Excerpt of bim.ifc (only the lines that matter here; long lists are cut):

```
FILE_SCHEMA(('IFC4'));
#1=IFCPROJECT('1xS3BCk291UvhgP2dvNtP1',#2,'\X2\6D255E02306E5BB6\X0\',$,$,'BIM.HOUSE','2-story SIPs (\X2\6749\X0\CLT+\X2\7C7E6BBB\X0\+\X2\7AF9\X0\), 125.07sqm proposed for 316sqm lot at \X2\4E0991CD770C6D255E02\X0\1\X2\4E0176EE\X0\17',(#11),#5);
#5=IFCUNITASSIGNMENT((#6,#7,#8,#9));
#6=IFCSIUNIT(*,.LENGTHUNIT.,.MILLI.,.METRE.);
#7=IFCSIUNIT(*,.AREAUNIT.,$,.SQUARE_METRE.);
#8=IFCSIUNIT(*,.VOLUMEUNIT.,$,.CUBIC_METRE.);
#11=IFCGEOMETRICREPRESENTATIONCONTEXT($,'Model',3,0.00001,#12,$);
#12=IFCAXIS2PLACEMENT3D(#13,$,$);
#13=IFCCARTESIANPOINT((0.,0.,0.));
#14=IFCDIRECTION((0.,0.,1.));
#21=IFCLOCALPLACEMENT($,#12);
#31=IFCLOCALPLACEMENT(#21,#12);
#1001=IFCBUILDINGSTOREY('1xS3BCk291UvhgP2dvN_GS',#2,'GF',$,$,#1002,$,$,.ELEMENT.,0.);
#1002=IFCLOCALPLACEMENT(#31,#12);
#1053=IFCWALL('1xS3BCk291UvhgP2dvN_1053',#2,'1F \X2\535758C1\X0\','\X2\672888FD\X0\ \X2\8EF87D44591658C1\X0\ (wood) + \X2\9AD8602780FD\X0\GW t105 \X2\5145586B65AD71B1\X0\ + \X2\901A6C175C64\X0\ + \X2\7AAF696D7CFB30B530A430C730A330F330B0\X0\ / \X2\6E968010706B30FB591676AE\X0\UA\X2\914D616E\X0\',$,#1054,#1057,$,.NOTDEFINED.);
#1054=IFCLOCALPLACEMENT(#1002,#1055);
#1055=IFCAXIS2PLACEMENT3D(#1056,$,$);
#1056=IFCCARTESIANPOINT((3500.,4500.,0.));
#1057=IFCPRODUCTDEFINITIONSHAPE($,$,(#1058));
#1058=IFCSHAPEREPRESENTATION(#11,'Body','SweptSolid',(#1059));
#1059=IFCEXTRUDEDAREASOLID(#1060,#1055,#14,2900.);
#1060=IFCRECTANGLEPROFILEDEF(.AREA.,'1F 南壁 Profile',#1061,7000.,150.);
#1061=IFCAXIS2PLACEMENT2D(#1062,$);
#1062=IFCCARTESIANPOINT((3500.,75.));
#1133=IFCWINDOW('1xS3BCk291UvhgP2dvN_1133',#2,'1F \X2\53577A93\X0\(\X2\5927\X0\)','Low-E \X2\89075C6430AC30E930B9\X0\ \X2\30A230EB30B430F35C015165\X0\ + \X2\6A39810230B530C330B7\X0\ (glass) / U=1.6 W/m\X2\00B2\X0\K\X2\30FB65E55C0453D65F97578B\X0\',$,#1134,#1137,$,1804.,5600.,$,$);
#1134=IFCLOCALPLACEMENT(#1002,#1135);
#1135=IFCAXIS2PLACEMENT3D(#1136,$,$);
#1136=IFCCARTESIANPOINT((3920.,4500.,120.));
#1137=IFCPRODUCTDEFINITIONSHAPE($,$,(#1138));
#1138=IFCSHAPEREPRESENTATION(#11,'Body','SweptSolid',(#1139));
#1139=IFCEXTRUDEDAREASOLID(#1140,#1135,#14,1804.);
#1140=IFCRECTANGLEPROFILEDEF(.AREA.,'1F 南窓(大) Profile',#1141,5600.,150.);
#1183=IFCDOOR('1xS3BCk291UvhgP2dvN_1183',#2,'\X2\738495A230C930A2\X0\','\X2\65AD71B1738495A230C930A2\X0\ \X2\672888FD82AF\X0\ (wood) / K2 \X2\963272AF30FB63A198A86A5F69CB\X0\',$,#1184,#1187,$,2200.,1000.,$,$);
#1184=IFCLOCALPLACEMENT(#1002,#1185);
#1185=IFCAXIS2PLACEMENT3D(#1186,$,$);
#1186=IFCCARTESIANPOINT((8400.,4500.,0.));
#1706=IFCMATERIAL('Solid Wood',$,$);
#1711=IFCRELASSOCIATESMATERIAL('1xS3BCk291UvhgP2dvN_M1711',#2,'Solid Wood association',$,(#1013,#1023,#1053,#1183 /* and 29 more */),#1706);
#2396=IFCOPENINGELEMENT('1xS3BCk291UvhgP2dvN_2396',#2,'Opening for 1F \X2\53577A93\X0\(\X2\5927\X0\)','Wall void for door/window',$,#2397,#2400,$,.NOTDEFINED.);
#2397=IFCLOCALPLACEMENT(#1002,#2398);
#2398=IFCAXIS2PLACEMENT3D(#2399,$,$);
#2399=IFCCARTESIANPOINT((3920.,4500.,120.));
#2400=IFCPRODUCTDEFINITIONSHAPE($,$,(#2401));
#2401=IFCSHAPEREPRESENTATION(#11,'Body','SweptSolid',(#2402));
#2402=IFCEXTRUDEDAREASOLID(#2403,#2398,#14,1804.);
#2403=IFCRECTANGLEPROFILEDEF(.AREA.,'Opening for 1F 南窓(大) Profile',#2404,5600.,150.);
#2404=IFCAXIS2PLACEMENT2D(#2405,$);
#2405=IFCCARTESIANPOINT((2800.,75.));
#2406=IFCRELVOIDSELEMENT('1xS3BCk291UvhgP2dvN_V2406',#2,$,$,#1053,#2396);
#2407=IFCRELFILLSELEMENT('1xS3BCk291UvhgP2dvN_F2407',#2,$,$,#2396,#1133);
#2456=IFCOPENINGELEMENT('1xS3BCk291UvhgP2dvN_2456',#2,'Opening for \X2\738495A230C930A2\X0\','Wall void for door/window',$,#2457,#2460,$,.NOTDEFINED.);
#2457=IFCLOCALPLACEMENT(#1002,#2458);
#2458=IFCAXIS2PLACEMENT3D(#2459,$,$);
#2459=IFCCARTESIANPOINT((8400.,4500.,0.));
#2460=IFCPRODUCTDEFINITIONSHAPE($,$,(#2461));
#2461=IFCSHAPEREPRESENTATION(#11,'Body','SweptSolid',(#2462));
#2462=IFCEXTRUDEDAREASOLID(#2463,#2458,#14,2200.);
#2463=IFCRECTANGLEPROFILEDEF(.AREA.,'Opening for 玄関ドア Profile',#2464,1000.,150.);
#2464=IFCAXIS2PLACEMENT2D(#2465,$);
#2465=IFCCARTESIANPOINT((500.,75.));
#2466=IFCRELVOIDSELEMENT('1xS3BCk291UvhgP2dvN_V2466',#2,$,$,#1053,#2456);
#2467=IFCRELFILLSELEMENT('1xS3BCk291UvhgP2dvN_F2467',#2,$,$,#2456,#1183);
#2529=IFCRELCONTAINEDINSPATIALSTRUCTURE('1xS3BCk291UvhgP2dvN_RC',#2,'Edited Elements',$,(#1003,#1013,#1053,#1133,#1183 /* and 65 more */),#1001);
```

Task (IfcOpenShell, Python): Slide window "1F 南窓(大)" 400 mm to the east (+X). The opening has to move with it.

```python
import ifcopenshell
import ifcopenshell.api.geometry
import ifcopenshell.util.placement
import ifcopenshell.util.unit

model = ifcopenshell.open("bim.ifc")
unit_scale = ifcopenshell.util.unit.calculate_unit_scale(model)

window = model.by_guid("1xS3BCk291UvhgP2dvN_1133")
opening = window.FillsVoids[0].RelatingOpeningElement
wall = opening.VoidsElements[0].RelatingBuildingElement

wall_matrix = ifcopenshell.util.placement.get_local_placement(wall.ObjectPlacement)
shift = wall_matrix[:3, 0] * 0.4 / unit_scale
before = ifcopenshell.util.placement.get_local_placement(window.ObjectPlacement)[:3, 3].copy()

# The window is not placed relative to its opening, so move both.
for product in (opening, window):
    matrix = ifcopenshell.util.placement.get_local_placement(product.ObjectPlacement)
    matrix[:3, 3] += shift
    ifcopenshell.api.geometry.edit_object_placement(model, product=product, matrix=matrix, is_si=False)

after = ifcopenshell.util.placement.get_local_placement(window.ObjectPlacement)[:3, 3]
print("window moved by", (after - before).round(3) + 0.0)

model.write("bim_edited.ifc")
```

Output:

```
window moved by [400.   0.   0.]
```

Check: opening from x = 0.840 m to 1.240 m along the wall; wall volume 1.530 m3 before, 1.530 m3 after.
